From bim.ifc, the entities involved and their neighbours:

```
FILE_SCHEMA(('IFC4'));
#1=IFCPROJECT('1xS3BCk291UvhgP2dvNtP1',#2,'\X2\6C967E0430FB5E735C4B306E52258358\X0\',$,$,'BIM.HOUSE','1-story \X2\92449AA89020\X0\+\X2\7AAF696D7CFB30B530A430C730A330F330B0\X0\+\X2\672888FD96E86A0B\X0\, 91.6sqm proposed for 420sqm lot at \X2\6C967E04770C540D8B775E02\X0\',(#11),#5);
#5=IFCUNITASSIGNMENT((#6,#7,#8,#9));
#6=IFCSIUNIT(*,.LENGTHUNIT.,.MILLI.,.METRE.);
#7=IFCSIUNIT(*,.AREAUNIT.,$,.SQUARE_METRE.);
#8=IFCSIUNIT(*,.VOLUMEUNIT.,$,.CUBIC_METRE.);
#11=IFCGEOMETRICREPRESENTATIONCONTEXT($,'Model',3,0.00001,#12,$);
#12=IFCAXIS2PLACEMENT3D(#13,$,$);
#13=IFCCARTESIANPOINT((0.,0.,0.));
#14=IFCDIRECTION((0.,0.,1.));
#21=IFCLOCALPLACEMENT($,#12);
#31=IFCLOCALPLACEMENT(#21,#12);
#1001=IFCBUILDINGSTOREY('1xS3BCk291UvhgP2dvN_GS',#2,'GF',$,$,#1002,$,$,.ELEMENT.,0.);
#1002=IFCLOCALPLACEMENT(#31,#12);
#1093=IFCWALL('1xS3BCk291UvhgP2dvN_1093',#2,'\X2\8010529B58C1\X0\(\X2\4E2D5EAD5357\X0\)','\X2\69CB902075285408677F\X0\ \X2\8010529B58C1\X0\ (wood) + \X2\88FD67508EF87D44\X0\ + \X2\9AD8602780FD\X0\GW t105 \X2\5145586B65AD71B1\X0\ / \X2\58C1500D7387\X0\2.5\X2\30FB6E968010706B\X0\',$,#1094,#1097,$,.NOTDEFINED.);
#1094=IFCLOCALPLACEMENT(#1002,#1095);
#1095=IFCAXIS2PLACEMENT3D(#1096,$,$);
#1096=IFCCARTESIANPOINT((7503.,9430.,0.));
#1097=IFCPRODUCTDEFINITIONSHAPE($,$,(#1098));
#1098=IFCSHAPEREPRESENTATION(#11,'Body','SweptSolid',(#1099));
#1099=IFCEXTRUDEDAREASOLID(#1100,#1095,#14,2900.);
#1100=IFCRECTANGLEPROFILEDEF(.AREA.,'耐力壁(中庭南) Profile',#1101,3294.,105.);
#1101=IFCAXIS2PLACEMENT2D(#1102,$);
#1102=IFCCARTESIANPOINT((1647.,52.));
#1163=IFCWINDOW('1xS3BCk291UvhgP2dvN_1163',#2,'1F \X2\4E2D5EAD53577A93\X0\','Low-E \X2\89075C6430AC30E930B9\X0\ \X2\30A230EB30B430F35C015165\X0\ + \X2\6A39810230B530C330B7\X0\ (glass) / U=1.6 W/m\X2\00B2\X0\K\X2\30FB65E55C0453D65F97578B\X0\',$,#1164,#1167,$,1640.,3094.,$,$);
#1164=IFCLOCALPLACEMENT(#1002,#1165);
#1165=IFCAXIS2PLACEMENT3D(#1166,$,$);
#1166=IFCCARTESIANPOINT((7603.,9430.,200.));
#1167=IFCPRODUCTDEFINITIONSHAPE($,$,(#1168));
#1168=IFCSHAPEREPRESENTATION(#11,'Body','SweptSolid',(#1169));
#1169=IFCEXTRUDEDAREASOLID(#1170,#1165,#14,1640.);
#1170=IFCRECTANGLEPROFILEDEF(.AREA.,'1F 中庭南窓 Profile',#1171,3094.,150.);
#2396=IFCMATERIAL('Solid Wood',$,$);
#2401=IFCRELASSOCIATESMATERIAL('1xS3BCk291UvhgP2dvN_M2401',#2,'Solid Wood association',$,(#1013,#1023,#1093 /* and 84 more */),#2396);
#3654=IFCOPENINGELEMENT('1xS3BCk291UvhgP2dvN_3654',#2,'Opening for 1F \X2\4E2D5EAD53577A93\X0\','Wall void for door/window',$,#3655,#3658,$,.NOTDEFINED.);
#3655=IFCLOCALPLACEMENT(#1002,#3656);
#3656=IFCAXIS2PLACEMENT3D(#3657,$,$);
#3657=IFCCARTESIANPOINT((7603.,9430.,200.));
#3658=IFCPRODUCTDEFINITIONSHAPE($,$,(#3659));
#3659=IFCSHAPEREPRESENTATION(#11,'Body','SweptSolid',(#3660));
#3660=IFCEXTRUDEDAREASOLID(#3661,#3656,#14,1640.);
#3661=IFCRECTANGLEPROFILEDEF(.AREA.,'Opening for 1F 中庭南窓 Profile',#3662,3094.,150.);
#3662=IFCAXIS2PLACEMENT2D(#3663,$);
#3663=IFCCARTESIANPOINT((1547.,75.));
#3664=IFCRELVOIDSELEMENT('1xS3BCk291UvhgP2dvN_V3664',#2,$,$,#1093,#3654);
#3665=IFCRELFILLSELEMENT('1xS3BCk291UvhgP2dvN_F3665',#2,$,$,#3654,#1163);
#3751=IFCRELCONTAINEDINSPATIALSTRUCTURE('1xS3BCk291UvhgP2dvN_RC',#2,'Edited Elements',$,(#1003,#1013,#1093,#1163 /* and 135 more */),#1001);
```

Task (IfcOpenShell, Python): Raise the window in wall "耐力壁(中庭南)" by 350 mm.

```python
import numpy as np
import ifcopenshell
import ifcopenshell.api.geometry
import ifcopenshell.util.placement
import ifcopenshell.util.unit

model = ifcopenshell.open("bim.ifc")
unit_scale = ifcopenshell.util.unit.calculate_unit_scale(model)

window = model.by_guid("1xS3BCk291UvhgP2dvN_1163")
opening = window.FillsVoids[0].RelatingOpeningElement
dz = 350.0

shift = np.array([0.0, 0.0, dz])
# The window is not placed relative to its opening, so move both.
for product in (opening, window):
    matrix = ifcopenshell.util.placement.get_local_placement(product.ObjectPlacement)
    matrix[:3, 3] += shift
    ifcopenshell.api.geometry.edit_object_placement(model, product=product, matrix=matrix, is_si=False)

print(f"moved by {dz * unit_scale:+.3f} m")

model.write("bim_updated.ifc")
```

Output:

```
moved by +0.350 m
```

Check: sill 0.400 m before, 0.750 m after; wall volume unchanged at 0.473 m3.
